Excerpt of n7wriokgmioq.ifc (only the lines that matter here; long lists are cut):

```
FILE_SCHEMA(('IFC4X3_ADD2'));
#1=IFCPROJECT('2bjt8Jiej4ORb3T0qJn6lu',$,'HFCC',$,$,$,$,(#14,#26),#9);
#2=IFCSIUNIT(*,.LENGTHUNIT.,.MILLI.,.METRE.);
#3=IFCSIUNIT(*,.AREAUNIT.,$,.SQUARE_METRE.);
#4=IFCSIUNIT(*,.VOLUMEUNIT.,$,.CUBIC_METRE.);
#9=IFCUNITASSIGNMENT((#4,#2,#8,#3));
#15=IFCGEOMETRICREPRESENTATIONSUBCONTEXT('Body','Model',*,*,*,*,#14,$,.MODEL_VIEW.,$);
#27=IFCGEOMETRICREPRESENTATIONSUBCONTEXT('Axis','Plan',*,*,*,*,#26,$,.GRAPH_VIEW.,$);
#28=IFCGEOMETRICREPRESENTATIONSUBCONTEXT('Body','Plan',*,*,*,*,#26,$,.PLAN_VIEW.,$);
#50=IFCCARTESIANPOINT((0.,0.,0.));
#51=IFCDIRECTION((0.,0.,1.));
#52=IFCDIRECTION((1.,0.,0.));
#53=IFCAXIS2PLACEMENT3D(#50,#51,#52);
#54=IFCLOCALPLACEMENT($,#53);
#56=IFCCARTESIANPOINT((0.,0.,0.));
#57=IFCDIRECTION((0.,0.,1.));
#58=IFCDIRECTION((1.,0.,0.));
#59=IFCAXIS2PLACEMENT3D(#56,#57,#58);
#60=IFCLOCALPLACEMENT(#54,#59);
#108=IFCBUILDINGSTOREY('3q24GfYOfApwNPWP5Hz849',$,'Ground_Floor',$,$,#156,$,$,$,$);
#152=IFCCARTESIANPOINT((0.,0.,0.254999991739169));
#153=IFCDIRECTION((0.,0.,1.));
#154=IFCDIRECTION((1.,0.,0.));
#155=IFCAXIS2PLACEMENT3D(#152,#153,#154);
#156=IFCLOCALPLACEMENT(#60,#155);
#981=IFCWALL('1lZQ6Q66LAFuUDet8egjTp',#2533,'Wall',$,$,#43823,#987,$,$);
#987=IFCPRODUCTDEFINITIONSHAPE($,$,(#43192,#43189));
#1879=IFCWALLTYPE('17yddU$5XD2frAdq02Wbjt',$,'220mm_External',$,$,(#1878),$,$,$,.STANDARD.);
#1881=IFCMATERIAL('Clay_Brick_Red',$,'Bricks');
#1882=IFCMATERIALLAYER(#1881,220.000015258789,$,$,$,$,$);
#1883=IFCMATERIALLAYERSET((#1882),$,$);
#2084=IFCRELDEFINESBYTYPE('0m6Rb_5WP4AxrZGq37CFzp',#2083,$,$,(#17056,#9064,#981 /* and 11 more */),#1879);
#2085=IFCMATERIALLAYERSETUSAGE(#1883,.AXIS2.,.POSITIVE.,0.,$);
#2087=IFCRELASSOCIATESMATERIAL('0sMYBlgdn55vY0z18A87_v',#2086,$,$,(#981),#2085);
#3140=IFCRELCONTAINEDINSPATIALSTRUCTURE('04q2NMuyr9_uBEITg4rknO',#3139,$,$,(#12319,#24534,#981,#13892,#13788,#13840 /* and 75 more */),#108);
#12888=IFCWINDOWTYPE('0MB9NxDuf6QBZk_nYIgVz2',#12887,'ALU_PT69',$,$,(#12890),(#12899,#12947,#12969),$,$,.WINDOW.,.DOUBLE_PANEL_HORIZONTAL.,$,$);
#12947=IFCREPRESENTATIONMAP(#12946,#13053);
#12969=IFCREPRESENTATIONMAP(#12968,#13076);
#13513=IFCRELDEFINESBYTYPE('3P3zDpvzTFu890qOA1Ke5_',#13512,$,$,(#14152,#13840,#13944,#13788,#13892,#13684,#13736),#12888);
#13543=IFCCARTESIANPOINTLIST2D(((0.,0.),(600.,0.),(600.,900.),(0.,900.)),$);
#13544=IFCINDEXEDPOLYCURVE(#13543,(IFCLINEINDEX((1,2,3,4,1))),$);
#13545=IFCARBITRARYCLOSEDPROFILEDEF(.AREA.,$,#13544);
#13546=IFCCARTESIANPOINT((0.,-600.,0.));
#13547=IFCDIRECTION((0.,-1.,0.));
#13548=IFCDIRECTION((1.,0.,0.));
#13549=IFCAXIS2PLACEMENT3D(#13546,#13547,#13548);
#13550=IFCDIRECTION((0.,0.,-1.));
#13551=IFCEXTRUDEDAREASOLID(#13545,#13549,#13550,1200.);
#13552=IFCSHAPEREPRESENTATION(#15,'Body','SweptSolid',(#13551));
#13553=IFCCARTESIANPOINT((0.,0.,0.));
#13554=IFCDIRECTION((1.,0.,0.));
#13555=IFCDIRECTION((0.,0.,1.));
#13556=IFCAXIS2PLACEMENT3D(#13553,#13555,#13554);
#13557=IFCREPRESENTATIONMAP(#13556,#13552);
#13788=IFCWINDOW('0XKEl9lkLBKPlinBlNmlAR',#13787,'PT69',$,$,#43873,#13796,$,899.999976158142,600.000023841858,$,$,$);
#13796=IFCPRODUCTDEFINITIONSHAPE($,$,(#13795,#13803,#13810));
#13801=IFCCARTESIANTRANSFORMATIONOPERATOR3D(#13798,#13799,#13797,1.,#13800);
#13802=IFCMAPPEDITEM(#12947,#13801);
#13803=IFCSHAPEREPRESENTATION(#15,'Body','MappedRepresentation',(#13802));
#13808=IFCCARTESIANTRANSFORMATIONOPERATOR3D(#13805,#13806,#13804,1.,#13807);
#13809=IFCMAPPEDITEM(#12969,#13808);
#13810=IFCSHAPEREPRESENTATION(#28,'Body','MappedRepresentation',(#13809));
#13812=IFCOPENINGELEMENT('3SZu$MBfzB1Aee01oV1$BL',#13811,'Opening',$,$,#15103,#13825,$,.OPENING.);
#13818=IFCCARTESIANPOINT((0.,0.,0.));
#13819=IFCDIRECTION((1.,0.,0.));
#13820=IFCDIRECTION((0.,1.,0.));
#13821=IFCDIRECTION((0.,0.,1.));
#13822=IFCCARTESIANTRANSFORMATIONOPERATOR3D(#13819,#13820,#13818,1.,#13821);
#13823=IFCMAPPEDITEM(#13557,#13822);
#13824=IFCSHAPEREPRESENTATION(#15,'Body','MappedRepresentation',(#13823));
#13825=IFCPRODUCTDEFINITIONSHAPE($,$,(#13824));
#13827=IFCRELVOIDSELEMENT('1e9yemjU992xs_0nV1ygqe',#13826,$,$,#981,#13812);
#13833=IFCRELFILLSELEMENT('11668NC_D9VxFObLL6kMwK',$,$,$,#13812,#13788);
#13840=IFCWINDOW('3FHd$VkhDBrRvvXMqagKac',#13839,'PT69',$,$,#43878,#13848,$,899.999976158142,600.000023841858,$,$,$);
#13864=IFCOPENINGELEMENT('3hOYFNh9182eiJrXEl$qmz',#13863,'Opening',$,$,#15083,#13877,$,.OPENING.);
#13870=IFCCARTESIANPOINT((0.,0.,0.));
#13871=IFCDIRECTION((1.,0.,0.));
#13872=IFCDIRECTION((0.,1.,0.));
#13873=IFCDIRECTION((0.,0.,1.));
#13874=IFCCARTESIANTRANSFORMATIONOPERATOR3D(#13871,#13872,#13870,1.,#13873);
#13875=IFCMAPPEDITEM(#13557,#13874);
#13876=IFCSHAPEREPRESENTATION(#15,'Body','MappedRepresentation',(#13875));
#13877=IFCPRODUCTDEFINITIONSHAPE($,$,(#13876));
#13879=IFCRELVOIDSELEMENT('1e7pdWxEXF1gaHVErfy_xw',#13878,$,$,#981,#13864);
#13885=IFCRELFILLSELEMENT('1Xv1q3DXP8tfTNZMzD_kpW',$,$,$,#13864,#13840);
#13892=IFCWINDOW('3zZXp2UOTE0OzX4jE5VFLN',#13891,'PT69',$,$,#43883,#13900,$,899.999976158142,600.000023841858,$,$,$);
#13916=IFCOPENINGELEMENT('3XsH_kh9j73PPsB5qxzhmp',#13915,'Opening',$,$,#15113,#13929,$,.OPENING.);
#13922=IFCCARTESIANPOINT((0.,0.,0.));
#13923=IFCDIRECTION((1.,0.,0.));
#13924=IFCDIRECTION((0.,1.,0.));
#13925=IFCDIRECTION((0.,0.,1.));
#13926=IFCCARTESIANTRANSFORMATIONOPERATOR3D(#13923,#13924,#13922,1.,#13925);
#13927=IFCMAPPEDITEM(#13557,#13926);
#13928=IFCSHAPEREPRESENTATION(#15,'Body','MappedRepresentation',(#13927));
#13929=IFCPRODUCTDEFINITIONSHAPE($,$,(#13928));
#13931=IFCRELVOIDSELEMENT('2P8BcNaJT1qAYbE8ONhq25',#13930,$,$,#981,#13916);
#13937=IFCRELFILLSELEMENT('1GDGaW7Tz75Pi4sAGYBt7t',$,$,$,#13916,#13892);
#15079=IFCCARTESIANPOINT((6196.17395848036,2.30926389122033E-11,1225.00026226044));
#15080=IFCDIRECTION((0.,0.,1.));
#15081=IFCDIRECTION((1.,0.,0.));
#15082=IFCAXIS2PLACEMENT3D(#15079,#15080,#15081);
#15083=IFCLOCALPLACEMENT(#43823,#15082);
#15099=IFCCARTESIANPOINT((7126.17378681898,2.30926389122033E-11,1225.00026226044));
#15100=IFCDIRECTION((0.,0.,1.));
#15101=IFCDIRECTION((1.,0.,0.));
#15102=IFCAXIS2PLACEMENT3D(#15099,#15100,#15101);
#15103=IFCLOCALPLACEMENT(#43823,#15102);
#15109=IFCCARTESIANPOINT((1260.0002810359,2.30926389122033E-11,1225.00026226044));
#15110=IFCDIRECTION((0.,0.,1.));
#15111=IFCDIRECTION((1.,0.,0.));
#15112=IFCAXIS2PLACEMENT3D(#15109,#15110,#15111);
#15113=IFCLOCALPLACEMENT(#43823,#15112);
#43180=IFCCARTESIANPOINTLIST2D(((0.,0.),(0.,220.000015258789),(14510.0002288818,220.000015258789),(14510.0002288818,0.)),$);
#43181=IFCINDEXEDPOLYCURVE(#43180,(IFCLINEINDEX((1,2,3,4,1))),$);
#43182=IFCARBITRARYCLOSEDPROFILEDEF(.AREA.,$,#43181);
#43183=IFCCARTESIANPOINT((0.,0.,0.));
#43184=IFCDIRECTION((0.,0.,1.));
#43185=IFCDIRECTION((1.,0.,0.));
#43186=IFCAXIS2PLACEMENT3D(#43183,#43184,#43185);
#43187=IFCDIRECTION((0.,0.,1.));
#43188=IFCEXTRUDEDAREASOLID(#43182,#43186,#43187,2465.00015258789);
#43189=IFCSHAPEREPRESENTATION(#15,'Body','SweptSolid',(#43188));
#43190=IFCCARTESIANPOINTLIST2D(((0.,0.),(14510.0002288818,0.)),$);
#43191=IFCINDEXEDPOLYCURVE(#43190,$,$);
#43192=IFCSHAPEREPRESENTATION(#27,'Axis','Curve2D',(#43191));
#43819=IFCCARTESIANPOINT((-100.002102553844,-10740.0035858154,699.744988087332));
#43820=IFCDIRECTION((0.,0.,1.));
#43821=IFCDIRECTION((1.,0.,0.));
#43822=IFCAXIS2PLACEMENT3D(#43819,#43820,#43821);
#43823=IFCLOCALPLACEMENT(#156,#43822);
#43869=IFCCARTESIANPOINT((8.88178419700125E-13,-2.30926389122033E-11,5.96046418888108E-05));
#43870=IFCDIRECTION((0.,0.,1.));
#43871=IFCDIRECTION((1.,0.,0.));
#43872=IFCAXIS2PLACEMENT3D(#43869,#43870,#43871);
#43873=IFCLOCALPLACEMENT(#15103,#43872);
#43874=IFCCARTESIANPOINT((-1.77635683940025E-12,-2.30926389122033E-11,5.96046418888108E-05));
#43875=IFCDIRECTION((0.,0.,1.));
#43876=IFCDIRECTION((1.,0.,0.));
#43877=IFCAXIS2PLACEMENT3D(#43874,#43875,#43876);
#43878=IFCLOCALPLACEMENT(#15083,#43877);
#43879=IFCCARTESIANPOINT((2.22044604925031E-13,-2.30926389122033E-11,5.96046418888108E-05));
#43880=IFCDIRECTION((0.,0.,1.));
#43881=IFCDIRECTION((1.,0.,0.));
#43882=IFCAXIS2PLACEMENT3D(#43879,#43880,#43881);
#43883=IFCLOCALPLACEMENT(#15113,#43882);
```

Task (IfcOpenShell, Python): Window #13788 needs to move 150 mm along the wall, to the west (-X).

```python
import ifcopenshell
import ifcopenshell.api.geometry
import ifcopenshell.util.placement
import ifcopenshell.util.unit

model = ifcopenshell.open("n7wriokgmioq.ifc")
unit_scale = ifcopenshell.util.unit.calculate_unit_scale(model)

window = model.by_id(13788)
opening = window.FillsVoids[0].RelatingOpeningElement
wall = opening.VoidsElements[0].RelatingBuildingElement

wall_matrix = ifcopenshell.util.placement.get_local_placement(wall.ObjectPlacement)
shift = wall_matrix[:3, 0] * -0.15 / unit_scale
before = ifcopenshell.util.placement.get_local_placement(window.ObjectPlacement)[:3, 3].copy()

# The window is placed relative to its opening, so it follows when the opening moves.
matrix = ifcopenshell.util.placement.get_local_placement(opening.ObjectPlacement)
matrix[:3, 3] += shift
ifcopenshell.api.geometry.edit_object_placement(
    model, product=opening, matrix=matrix, is_si=False, should_transform_children=True
)

after = ifcopenshell.util.placement.get_local_placement(window.ObjectPlacement)[:3, 3]
print("window moved by", (after - before).round(3) + 0.0)

model.write("n7wriokgmioq_updated.ifc")
```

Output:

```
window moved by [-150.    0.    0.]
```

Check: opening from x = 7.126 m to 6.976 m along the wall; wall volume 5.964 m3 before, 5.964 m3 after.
